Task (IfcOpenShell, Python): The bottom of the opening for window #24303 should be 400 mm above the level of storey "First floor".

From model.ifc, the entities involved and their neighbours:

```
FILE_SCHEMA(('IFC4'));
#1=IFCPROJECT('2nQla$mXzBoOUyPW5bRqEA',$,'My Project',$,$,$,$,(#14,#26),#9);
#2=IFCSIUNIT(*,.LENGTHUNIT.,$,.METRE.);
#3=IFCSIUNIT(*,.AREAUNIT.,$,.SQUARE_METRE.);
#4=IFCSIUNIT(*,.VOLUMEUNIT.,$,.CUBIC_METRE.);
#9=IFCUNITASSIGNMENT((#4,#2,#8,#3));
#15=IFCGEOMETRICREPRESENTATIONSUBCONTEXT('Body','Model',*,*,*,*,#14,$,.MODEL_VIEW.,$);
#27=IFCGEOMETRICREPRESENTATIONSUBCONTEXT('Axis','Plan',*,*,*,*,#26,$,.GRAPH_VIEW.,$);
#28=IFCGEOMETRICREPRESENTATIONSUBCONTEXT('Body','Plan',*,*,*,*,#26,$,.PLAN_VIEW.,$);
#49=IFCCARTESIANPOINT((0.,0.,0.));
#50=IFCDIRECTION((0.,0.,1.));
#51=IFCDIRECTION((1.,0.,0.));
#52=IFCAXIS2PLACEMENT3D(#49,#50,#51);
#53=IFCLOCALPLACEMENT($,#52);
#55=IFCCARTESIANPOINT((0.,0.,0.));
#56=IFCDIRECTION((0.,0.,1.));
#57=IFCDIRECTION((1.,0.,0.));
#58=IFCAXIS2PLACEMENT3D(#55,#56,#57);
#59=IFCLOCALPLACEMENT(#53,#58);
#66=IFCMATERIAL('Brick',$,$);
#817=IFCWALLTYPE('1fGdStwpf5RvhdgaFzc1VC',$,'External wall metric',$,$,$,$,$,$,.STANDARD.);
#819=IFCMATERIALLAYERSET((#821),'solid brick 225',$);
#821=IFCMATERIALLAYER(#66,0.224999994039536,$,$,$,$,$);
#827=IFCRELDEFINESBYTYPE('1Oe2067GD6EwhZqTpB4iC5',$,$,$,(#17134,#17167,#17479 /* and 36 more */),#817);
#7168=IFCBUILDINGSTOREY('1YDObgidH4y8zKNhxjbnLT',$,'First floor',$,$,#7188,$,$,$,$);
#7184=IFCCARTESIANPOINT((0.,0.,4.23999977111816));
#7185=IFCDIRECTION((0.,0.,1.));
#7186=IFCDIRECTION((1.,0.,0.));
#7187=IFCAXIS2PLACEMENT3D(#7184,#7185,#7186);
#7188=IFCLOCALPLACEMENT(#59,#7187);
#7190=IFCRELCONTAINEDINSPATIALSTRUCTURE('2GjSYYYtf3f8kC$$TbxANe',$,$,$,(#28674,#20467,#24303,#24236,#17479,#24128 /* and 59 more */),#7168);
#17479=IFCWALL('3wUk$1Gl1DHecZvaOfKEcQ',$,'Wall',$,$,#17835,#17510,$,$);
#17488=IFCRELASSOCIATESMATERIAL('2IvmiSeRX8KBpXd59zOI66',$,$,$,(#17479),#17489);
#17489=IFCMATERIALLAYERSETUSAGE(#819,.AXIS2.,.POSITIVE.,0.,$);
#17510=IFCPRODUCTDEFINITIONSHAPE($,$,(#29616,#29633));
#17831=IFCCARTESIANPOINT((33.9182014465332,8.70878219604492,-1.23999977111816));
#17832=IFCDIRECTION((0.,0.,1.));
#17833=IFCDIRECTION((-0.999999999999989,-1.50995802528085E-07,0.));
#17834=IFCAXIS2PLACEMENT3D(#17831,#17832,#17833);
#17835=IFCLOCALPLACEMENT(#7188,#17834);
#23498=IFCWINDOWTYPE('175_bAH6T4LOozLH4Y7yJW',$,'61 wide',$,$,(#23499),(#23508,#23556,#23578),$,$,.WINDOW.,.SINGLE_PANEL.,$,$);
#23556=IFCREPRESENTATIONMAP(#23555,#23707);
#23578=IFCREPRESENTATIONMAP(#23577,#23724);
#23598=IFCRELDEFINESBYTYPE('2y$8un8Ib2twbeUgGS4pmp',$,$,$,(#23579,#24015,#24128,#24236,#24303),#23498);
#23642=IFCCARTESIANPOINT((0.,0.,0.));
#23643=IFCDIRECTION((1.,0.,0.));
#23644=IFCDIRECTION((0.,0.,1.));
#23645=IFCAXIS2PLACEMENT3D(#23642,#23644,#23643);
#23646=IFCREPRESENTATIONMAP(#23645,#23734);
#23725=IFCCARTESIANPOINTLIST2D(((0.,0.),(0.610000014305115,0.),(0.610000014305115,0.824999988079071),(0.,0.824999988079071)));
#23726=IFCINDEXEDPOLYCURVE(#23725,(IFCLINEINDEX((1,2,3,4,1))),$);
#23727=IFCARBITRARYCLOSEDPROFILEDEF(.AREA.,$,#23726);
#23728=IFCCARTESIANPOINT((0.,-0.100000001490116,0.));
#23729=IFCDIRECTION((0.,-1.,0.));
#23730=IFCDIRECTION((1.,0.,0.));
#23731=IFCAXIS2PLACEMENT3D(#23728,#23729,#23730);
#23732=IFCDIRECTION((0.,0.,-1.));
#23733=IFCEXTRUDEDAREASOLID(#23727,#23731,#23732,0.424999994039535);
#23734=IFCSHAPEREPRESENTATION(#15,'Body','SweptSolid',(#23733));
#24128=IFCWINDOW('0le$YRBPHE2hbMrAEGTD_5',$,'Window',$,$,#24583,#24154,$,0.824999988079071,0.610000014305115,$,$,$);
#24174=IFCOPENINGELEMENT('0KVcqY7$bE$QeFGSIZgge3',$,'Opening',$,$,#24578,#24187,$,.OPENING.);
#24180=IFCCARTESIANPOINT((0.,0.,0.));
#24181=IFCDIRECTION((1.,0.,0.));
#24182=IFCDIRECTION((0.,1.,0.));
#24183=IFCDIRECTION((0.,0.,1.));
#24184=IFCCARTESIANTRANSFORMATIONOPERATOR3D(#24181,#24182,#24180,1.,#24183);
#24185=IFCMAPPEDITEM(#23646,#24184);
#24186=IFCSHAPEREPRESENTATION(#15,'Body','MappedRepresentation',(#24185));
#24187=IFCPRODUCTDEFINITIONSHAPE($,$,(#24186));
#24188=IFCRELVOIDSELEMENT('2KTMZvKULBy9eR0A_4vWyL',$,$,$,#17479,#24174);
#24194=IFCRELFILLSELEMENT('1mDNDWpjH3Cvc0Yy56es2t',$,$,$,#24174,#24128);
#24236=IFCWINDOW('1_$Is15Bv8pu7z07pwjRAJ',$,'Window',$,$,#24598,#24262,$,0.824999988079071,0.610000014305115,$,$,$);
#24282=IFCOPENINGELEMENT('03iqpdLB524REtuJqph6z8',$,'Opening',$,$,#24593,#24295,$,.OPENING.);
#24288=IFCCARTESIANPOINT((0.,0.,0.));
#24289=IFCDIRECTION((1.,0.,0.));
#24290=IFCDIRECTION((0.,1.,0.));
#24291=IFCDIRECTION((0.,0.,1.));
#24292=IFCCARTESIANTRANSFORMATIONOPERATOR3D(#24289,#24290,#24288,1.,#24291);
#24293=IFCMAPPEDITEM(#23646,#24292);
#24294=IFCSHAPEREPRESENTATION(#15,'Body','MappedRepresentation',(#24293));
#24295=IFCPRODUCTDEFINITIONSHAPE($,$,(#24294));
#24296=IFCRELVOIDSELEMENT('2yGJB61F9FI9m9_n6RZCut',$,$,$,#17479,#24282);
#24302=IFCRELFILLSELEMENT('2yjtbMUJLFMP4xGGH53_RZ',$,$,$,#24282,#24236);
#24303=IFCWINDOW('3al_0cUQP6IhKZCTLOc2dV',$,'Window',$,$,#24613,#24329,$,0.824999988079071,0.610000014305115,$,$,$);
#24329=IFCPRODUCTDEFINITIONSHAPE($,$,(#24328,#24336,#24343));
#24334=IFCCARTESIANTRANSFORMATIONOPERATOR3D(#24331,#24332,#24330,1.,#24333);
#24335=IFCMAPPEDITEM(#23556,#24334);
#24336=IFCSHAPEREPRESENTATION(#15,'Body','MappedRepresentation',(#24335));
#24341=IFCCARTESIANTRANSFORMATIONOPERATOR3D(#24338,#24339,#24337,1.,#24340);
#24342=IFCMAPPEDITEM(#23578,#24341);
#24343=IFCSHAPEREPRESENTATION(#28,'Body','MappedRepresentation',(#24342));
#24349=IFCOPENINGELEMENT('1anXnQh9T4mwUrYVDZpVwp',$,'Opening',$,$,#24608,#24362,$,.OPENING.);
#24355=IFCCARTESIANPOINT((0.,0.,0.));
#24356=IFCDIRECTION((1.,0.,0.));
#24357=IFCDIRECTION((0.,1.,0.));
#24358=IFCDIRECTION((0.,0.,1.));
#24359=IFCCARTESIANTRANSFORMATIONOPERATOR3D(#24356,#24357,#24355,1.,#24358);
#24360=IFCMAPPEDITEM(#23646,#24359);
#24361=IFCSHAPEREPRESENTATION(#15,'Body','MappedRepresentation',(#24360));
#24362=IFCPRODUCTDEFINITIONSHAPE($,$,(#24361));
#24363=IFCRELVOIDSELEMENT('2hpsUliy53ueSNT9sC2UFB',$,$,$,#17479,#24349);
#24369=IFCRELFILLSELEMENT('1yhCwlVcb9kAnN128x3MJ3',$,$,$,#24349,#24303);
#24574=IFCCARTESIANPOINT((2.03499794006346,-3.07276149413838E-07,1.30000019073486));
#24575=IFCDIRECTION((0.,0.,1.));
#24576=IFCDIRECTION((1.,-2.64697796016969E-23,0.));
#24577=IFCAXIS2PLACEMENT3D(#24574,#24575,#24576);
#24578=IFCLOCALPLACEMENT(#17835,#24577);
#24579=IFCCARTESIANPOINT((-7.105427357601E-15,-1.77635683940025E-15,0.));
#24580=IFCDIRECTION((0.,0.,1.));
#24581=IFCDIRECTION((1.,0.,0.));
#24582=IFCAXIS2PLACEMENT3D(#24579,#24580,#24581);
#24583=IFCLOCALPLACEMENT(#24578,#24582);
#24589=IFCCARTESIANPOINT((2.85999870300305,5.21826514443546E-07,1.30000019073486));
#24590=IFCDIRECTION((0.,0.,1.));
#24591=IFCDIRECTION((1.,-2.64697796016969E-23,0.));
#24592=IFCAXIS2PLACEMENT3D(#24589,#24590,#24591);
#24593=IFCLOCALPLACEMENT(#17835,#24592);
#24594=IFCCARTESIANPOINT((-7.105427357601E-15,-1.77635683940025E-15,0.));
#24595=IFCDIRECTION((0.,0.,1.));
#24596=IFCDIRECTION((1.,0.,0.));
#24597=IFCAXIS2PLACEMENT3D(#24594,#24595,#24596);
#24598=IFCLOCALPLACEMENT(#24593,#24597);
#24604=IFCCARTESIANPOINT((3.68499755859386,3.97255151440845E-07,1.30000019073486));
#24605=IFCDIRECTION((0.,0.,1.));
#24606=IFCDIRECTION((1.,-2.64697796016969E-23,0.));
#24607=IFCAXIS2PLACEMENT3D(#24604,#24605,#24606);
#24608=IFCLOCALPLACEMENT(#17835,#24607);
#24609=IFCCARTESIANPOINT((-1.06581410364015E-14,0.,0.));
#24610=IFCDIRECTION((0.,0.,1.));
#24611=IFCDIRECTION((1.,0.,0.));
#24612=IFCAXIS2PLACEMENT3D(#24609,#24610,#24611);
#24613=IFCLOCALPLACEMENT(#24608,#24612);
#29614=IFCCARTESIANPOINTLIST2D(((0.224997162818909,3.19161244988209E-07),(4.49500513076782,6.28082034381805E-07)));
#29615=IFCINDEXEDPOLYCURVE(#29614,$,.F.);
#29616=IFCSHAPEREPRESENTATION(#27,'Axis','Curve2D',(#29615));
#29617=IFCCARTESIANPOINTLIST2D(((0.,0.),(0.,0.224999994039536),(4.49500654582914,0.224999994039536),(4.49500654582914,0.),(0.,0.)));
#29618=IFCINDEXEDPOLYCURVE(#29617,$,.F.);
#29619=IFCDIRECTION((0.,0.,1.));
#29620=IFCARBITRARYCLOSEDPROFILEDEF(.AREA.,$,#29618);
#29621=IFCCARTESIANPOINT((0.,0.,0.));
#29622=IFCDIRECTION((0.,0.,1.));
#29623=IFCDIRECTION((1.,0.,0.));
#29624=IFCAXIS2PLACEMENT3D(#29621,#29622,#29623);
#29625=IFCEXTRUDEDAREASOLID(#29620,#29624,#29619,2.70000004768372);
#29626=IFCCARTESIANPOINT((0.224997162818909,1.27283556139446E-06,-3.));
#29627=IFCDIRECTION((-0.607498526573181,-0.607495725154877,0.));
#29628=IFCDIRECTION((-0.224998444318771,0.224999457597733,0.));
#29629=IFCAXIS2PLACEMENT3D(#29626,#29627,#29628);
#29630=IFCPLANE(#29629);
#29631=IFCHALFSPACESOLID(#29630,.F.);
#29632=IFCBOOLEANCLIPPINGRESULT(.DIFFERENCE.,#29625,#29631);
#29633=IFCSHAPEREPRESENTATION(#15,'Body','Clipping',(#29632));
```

```python
import numpy as np
import ifcopenshell
import ifcopenshell.api.geometry
import ifcopenshell.geom
import ifcopenshell.util.element
import ifcopenshell.util.placement
import ifcopenshell.util.shape
import ifcopenshell.util.unit

model = ifcopenshell.open("model.ifc")
unit_scale = ifcopenshell.util.unit.calculate_unit_scale(model)

window = model.by_id(24303)
opening = window.FillsVoids[0].RelatingOpeningElement
storey = ifcopenshell.util.element.get_container(window, ifc_class="IfcBuildingStorey")
level = ifcopenshell.util.placement.get_local_placement(storey.ObjectPlacement)[2, 3]

# The opening's origin need not be at the sill, so measure its lowest point.
shape = ifcopenshell.geom.create_shape(ifcopenshell.geom.settings(), opening)
bottom = ifcopenshell.util.shape.get_shape_bottom_elevation(shape, shape.geometry) / unit_scale
dz = level + 0.4 / unit_scale - bottom

shift = np.array([0.0, 0.0, dz])
# The window is placed relative to its opening, so it follows when the opening moves.
matrix = ifcopenshell.util.placement.get_local_placement(opening.ObjectPlacement)
matrix[:3, 3] += shift
ifcopenshell.api.geometry.edit_object_placement(
    model, product=opening, matrix=matrix, is_si=False, should_transform_children=True
)

print(f"moved by {dz * unit_scale:+.3f} m")

model.write("model_updated.ifc")
```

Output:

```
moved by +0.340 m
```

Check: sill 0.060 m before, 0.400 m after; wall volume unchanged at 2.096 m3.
